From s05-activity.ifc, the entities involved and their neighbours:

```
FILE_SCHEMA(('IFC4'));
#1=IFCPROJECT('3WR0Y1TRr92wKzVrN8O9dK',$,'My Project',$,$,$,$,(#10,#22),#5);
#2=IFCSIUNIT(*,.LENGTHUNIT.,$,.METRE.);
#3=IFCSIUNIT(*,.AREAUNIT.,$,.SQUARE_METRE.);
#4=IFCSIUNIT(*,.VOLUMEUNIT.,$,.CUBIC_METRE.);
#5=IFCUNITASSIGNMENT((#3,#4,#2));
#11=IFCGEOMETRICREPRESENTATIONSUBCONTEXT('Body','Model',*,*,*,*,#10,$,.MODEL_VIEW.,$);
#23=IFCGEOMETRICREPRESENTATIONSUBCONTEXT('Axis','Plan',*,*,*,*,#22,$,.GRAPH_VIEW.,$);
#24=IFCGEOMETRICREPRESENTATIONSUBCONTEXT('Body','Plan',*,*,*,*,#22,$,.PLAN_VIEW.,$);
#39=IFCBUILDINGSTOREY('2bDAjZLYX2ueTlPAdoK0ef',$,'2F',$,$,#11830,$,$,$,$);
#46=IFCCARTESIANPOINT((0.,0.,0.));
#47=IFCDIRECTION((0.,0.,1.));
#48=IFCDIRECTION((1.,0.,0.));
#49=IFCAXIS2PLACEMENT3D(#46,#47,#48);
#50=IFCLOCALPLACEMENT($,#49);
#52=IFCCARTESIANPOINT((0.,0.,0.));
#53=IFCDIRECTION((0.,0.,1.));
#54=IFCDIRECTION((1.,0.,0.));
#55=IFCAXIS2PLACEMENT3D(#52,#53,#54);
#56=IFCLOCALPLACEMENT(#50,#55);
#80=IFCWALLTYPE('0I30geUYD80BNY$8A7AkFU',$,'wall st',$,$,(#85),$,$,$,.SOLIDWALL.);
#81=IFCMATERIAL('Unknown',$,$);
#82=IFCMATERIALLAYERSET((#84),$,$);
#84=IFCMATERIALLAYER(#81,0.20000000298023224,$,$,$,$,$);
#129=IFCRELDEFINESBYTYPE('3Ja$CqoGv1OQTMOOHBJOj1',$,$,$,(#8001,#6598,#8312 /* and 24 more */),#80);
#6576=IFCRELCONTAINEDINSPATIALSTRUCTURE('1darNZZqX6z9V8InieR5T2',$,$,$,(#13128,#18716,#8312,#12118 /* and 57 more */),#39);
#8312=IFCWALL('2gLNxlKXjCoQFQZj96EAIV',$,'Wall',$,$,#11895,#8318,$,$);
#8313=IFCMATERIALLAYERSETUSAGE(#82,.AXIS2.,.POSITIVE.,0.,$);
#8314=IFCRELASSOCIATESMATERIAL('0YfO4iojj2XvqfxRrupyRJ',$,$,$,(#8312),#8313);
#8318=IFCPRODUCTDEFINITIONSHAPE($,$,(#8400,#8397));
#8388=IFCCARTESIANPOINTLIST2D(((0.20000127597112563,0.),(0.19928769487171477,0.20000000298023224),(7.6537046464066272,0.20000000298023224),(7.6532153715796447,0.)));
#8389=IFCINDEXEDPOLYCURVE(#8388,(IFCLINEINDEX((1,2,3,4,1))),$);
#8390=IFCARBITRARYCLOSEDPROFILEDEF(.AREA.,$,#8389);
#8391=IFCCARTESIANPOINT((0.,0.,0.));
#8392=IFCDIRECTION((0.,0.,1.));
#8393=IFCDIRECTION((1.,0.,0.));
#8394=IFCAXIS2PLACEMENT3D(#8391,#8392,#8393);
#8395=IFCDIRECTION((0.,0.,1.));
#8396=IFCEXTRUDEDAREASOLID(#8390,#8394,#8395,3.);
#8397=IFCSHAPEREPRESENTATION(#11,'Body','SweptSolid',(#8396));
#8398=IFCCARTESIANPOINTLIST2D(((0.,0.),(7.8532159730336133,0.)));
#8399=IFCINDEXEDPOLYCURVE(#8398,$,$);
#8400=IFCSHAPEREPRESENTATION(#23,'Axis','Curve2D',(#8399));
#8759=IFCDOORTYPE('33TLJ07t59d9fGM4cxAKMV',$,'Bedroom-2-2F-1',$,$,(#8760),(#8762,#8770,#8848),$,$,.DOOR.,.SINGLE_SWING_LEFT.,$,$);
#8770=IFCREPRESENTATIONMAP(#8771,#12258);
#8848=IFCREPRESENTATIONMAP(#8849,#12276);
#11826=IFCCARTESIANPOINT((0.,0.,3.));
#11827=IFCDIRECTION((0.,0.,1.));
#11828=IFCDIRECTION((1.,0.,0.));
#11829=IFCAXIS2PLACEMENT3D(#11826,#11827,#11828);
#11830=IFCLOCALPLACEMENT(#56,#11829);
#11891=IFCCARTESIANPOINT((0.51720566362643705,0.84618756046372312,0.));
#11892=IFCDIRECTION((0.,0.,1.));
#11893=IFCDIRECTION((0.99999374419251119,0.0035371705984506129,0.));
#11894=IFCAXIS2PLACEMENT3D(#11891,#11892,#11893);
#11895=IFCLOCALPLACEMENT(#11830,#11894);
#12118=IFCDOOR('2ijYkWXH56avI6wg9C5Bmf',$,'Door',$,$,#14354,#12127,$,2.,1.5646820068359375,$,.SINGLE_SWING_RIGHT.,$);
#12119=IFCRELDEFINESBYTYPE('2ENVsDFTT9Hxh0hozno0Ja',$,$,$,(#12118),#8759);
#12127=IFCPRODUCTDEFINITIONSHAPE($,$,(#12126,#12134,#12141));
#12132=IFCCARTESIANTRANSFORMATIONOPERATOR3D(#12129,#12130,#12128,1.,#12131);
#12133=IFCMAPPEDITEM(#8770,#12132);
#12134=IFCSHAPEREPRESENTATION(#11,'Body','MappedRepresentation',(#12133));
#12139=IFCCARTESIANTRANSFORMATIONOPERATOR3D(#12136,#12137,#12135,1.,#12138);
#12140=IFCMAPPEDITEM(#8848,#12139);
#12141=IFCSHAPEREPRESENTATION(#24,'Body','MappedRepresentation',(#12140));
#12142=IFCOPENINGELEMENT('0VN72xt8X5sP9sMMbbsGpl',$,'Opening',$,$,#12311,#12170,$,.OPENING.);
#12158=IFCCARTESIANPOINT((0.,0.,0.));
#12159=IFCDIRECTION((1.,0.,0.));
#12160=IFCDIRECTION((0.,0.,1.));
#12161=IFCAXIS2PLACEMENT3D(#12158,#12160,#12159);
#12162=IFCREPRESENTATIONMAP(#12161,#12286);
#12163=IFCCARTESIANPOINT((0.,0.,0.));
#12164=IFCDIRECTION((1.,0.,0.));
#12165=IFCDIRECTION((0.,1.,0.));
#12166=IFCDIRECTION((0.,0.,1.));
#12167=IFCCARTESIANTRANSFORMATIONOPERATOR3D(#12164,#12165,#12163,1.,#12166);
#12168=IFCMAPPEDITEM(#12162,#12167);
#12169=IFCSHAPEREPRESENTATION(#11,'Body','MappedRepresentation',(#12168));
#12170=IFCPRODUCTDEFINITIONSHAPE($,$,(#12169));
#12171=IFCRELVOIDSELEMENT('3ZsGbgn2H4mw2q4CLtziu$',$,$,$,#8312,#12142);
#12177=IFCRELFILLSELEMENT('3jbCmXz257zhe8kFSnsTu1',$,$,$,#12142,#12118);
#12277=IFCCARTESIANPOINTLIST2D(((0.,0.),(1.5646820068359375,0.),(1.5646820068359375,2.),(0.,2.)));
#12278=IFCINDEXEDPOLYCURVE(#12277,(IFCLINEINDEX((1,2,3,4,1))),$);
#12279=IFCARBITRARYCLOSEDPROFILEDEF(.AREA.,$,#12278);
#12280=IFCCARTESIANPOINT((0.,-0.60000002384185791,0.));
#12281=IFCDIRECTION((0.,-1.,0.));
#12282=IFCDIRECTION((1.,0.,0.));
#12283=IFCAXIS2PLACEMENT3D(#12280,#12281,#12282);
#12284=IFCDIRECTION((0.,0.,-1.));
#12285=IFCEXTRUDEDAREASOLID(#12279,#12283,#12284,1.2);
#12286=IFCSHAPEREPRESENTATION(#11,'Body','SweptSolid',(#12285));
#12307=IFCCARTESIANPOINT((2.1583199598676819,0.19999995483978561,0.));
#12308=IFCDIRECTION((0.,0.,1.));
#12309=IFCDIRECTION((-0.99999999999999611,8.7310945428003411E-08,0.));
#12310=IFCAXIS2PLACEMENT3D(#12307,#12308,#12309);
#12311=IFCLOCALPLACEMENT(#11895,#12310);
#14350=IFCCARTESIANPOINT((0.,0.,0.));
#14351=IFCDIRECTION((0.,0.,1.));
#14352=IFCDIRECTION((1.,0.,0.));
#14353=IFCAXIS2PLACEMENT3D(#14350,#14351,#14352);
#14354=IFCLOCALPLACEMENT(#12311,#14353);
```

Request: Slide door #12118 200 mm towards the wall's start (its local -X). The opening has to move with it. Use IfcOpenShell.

```python
import ifcopenshell
import ifcopenshell.api.geometry
import ifcopenshell.util.placement
import ifcopenshell.util.unit

model = ifcopenshell.open("s05-activity.ifc")
unit_scale = ifcopenshell.util.unit.calculate_unit_scale(model)

door = model.by_guid("2ijYkWXH56avI6wg9C5Bmf")
opening = door.FillsVoids[0].RelatingOpeningElement
wall = opening.VoidsElements[0].RelatingBuildingElement

wall_matrix = ifcopenshell.util.placement.get_local_placement(wall.ObjectPlacement)
shift = wall_matrix[:3, 0] * -0.2 / unit_scale
before = ifcopenshell.util.placement.get_local_placement(door.ObjectPlacement)[:3, 3].copy()

# The door is placed relative to its opening, so it follows when the opening moves.
matrix = ifcopenshell.util.placement.get_local_placement(opening.ObjectPlacement)
matrix[:3, 3] += shift
ifcopenshell.api.geometry.edit_object_placement(
    model, product=opening, matrix=matrix, is_si=False, should_transform_children=True
)

after = ifcopenshell.util.placement.get_local_placement(door.ObjectPlacement)[:3, 3]
print("door moved by", (after - before).round(3) + 0.0)

model.write("s05-activity_rev.ifc")
```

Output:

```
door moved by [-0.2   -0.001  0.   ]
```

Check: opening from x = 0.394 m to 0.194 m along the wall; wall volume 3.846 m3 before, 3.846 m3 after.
